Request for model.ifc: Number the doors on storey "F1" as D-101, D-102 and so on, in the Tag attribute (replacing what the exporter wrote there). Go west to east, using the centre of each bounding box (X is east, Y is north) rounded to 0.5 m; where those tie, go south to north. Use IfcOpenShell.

First a look at what the model holds.

```python
import ifcopenshell
import ifcopenshell.util.element
import ifcopenshell.util.placement

model = ifcopenshell.open("model.ifc")
print(model.schema)
storey = next(s for s in model.by_type("IfcBuildingStorey") if s.Name == "F1")
doors = [e for e in ifcopenshell.util.element.get_decomposition(storey) if e.is_a("IfcDoor")]
for e in sorted(doors, key=lambda e: e.id()):
    origin = ifcopenshell.util.placement.get_local_placement(e.ObjectPlacement)[:3, 3]
    print(e.id(), e.Tag, e.Name, origin.round(2) + 0.0, sep=" | ")
```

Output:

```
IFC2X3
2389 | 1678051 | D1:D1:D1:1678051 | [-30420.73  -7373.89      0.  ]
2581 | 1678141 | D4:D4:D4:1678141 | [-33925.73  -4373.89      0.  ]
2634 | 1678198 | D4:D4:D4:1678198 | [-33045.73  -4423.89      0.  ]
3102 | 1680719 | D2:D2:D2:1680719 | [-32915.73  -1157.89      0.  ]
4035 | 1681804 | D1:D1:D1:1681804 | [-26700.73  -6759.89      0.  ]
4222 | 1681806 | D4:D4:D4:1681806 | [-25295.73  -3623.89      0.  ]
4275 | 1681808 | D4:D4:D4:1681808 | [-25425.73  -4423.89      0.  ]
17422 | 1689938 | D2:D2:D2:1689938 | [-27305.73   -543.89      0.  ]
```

```python
import ifcopenshell
import ifcopenshell.geom
import ifcopenshell.util.element
import ifcopenshell.util.shape

model = ifcopenshell.open("model.ifc")
settings = ifcopenshell.geom.settings()
settings.set("use-world-coords", True)


def centre(element):
    shape = ifcopenshell.geom.create_shape(settings, element)
    return ifcopenshell.util.shape.get_bbox_centroid(shape.geometry)


storey = next(s for s in model.by_type("IfcBuildingStorey") if s.Name == "F1")
doors = [e for e in ifcopenshell.util.element.get_decomposition(storey) if e.is_a("IfcDoor")]

# Insertion points can sit at a corner or the storey origin, so sort by the geometry (in metres).
centres = {e: centre(e) for e in doors}
doors.sort(key=lambda e: (round(centres[e][0] / 0.5), centres[e][1]))

for i, e in enumerate(doors, start=1):
    number = f"D-1{i:02d}"
    e.Tag = number
    print(e.id(), number)

model.write("model_edited.ifc")
```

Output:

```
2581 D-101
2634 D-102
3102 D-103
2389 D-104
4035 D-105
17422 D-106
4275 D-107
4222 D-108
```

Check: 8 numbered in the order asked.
